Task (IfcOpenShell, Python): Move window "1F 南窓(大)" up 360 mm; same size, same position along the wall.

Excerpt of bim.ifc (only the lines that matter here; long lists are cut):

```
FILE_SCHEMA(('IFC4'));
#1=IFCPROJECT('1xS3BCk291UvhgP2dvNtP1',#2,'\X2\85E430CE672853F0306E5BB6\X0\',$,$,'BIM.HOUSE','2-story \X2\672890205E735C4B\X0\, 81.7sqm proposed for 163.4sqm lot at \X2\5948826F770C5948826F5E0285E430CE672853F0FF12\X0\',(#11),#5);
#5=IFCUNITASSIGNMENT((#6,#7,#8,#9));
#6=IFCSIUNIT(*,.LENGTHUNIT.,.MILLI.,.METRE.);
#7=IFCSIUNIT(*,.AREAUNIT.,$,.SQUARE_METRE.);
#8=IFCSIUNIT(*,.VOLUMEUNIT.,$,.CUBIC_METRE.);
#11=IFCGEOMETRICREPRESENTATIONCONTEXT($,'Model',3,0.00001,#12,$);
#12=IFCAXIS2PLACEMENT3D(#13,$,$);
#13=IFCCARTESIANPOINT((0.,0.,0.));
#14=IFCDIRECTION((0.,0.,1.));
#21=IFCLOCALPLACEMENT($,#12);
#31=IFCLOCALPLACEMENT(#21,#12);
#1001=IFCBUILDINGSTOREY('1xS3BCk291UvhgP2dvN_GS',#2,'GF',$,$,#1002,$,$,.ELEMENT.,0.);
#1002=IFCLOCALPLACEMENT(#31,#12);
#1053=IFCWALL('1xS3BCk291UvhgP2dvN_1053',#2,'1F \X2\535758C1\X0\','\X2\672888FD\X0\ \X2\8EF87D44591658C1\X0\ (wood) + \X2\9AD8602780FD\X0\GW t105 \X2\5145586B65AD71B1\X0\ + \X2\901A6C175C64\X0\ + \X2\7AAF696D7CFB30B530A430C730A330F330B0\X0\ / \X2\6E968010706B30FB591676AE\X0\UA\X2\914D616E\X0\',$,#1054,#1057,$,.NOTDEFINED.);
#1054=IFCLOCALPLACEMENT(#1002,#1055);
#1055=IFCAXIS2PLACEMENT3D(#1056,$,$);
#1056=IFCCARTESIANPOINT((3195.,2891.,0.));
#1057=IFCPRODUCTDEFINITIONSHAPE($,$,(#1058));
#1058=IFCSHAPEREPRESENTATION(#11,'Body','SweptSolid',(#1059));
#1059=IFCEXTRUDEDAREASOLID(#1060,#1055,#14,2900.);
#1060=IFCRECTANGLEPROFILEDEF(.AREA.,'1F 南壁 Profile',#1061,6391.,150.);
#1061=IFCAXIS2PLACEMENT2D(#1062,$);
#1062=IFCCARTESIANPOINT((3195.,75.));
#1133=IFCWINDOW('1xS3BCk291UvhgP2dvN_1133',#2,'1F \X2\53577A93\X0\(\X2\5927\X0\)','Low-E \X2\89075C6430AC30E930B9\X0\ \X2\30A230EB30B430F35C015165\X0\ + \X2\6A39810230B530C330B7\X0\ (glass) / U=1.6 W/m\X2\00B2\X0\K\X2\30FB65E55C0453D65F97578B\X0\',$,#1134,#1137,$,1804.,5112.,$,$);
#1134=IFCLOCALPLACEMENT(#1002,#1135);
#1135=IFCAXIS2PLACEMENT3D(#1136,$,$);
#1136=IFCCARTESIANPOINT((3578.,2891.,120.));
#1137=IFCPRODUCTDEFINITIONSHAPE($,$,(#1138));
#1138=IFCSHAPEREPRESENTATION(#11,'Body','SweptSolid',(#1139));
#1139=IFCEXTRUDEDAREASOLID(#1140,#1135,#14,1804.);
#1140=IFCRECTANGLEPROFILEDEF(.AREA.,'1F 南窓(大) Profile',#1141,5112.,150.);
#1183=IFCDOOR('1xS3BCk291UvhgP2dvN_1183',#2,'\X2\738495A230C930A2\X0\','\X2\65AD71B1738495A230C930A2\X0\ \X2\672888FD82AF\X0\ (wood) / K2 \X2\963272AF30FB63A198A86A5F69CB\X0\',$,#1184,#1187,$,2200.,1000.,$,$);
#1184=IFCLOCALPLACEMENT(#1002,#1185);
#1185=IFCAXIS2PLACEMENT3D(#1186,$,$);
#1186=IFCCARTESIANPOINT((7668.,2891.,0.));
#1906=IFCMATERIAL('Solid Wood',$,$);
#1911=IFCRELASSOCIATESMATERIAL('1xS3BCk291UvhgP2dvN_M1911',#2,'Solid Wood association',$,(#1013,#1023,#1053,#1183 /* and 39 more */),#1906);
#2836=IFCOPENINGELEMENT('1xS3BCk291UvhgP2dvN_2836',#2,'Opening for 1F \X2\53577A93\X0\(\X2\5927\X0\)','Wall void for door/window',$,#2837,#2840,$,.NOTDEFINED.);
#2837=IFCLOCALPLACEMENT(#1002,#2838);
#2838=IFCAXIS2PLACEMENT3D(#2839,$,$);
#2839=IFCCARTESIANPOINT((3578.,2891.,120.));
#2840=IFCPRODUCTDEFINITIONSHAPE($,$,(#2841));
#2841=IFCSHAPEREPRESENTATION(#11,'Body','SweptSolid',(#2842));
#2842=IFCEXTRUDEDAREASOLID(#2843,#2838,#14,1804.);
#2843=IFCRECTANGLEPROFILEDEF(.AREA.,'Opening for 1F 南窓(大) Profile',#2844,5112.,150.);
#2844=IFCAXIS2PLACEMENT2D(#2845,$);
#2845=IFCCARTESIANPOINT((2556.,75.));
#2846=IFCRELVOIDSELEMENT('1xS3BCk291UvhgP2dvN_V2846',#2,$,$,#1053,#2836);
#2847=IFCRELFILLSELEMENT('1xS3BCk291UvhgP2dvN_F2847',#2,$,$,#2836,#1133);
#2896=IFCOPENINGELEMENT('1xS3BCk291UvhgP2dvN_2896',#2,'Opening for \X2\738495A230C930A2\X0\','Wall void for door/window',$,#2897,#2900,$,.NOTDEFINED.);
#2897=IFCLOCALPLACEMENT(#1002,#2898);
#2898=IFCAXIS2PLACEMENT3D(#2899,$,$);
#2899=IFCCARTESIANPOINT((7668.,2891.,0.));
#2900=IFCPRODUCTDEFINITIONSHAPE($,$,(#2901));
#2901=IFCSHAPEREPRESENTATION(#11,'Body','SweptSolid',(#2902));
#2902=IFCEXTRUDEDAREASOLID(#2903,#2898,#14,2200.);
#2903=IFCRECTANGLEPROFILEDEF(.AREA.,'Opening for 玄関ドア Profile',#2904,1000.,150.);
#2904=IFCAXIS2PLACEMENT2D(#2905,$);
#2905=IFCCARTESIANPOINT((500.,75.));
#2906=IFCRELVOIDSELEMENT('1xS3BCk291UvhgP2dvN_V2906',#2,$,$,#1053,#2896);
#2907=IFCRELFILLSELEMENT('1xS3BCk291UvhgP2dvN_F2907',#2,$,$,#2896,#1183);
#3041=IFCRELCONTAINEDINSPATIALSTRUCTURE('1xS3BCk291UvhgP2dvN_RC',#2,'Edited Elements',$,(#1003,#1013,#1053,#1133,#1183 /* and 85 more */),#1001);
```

```python
import numpy as np
import ifcopenshell
import ifcopenshell.api.geometry
import ifcopenshell.util.placement
import ifcopenshell.util.unit

model = ifcopenshell.open("bim.ifc")
unit_scale = ifcopenshell.util.unit.calculate_unit_scale(model)

window = model.by_guid("1xS3BCk291UvhgP2dvN_1133")
opening = window.FillsVoids[0].RelatingOpeningElement
dz = 360.0

shift = np.array([0.0, 0.0, dz])
# The window is not placed relative to its opening, so move both.
for product in (opening, window):
    matrix = ifcopenshell.util.placement.get_local_placement(product.ObjectPlacement)
    matrix[:3, 3] += shift
    ifcopenshell.api.geometry.edit_object_placement(model, product=product, matrix=matrix, is_si=False)

print(f"moved by {dz * unit_scale:+.3f} m")

model.write("bim_edited.ifc")
```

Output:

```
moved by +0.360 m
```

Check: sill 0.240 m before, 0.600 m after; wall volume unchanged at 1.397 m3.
